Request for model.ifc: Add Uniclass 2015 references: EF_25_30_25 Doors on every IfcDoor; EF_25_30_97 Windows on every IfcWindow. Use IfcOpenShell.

First a look at what the model holds.

```python
import ifcopenshell

model = ifcopenshell.open("model.ifc")
print(model.schema)
print("classifications:", [c.Name for c in model.by_type("IfcClassification")])
for ifc_class in ("IfcDoor", "IfcRoof", "IfcStair", "IfcWall", "IfcWindow"):
    print(ifc_class, len(model.by_type(ifc_class)))
```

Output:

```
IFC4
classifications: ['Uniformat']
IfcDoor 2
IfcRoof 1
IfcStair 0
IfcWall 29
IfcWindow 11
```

```python
import ifcopenshell
import ifcopenshell.api.classification

model = ifcopenshell.open("model.ifc")

system = ifcopenshell.api.classification.add_classification(model, classification="Uniclass 2015")

codes = {
    "IfcDoor": ("EF_25_30_25", "Doors"),
    "IfcWindow": ("EF_25_30_97", "Windows"),
}
for ifc_class, (code, name) in codes.items():
    products = model.by_type(ifc_class)
    ifcopenshell.api.classification.add_reference(
        model, products=products, classification=system, identification=code, name=name
    )
    print(code, len(products))

model.write("model_rev.ifc")
```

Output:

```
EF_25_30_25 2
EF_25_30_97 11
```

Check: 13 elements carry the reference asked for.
